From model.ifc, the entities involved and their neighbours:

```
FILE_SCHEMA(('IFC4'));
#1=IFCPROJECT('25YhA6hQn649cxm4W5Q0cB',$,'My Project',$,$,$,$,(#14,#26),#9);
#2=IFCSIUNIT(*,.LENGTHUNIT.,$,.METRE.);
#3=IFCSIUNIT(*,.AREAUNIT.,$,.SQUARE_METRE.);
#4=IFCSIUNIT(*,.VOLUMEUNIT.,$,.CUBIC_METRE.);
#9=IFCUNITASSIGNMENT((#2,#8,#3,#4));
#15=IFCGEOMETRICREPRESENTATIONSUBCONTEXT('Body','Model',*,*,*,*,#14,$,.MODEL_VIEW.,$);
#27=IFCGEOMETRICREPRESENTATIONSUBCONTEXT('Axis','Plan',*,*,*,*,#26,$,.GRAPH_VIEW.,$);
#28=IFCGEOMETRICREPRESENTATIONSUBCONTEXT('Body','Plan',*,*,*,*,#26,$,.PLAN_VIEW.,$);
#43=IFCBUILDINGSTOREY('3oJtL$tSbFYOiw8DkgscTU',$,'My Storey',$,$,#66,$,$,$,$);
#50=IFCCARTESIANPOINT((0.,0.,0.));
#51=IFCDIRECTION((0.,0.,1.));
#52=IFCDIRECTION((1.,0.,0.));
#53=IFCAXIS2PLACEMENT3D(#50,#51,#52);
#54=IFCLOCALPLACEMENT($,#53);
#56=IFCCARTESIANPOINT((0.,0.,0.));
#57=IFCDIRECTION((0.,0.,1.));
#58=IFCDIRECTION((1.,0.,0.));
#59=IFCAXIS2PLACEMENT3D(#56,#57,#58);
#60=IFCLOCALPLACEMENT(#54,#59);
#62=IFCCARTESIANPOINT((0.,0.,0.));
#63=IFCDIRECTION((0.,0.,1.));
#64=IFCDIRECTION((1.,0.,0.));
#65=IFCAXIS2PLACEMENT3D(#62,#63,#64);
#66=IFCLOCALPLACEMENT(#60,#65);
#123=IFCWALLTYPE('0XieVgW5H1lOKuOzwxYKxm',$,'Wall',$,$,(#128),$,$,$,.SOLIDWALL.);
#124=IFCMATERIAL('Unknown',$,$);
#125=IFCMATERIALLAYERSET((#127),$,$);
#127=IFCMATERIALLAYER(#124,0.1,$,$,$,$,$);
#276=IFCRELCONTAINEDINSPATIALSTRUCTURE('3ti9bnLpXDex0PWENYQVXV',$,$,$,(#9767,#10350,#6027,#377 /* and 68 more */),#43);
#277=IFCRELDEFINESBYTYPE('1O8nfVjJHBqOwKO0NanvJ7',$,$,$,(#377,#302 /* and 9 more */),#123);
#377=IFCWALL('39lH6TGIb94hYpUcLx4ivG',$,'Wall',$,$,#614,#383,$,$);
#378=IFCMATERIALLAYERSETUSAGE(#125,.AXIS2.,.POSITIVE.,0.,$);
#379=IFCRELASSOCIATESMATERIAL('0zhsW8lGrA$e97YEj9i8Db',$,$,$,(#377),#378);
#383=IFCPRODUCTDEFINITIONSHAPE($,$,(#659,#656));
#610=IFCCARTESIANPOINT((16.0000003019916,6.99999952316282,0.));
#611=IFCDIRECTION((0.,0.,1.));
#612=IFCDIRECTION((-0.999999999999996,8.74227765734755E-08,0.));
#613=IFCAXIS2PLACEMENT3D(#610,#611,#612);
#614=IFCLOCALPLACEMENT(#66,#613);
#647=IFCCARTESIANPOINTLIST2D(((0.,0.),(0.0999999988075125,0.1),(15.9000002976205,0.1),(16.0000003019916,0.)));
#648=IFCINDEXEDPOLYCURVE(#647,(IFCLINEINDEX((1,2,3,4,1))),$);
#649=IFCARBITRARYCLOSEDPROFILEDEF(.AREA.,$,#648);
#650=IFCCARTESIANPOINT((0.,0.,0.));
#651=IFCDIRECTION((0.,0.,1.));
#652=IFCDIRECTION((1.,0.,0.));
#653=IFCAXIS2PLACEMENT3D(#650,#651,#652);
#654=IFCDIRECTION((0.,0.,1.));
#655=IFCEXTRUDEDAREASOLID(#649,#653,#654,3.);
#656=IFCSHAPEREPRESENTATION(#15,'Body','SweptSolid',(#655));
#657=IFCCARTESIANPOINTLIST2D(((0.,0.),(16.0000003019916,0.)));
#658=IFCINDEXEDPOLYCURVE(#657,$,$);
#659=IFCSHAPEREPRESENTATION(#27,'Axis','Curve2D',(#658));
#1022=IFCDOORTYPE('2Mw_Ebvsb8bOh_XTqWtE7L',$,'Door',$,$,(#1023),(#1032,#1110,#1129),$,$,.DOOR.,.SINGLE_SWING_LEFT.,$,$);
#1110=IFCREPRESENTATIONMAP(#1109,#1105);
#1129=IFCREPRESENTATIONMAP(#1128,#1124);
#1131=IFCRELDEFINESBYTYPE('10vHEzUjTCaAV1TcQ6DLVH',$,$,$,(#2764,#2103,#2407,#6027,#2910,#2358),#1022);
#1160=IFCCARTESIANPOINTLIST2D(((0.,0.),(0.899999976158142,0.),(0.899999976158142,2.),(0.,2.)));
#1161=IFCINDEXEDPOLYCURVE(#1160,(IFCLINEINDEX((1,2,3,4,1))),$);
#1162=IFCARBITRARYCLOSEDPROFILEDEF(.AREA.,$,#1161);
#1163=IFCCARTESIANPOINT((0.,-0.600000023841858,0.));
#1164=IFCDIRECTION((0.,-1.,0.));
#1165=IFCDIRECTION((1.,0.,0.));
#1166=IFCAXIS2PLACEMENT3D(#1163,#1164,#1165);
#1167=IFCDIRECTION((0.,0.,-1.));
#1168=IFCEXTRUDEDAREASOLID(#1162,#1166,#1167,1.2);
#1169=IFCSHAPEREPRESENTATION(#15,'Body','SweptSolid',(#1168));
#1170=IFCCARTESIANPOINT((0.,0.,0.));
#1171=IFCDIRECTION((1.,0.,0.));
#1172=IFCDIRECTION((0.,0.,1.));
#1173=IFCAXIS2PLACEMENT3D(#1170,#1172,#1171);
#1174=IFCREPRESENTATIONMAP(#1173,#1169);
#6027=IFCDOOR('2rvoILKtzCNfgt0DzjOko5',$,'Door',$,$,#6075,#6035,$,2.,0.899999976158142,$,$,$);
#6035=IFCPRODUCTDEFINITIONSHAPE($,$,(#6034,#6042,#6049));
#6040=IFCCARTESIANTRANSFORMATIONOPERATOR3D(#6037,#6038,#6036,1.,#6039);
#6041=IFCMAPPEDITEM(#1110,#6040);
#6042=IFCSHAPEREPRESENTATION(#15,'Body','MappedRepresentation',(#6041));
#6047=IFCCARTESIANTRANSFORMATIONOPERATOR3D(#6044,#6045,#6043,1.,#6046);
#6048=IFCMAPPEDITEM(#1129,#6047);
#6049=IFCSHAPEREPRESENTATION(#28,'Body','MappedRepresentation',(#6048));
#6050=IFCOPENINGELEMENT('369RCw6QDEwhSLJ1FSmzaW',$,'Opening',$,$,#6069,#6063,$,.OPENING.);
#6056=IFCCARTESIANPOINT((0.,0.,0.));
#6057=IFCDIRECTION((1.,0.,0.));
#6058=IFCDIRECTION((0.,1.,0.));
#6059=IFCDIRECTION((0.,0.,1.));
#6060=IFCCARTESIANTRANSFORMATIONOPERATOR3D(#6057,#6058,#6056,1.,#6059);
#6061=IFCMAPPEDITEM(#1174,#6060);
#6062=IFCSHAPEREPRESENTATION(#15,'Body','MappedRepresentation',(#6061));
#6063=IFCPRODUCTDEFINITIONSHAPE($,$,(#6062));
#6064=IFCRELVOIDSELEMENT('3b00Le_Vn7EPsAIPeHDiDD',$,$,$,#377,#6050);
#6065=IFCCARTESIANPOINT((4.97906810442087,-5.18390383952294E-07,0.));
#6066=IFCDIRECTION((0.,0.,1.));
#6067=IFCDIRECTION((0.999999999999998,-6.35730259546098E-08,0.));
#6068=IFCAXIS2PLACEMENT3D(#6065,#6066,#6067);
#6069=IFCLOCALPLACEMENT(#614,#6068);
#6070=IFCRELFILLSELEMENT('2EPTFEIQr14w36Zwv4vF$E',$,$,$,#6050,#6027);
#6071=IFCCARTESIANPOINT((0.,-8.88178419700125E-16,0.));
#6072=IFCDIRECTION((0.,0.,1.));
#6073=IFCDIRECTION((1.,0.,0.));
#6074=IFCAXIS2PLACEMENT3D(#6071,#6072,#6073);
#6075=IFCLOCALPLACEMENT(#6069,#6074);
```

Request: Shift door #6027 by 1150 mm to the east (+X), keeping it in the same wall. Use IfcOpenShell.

```python
import ifcopenshell
import ifcopenshell.api.geometry
import ifcopenshell.util.placement
import ifcopenshell.util.unit

model = ifcopenshell.open("model.ifc")
unit_scale = ifcopenshell.util.unit.calculate_unit_scale(model)

door = model.by_id(6027)
opening = door.FillsVoids[0].RelatingOpeningElement
wall = opening.VoidsElements[0].RelatingBuildingElement

wall_matrix = ifcopenshell.util.placement.get_local_placement(wall.ObjectPlacement)
shift = wall_matrix[:3, 0] * -1.15 / unit_scale
before = ifcopenshell.util.placement.get_local_placement(door.ObjectPlacement)[:3, 3].copy()

# The door is placed relative to its opening, so it follows when the opening moves.
matrix = ifcopenshell.util.placement.get_local_placement(opening.ObjectPlacement)
matrix[:3, 3] += shift
ifcopenshell.api.geometry.edit_object_placement(
    model, product=opening, matrix=matrix, is_si=False, should_transform_children=True
)

after = ifcopenshell.util.placement.get_local_placement(door.ObjectPlacement)[:3, 3]
print("door moved by", (after - before).round(3) + 0.0)

model.write("model-out.ifc")
```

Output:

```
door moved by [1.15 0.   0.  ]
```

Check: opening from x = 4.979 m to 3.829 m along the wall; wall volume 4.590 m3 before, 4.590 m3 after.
